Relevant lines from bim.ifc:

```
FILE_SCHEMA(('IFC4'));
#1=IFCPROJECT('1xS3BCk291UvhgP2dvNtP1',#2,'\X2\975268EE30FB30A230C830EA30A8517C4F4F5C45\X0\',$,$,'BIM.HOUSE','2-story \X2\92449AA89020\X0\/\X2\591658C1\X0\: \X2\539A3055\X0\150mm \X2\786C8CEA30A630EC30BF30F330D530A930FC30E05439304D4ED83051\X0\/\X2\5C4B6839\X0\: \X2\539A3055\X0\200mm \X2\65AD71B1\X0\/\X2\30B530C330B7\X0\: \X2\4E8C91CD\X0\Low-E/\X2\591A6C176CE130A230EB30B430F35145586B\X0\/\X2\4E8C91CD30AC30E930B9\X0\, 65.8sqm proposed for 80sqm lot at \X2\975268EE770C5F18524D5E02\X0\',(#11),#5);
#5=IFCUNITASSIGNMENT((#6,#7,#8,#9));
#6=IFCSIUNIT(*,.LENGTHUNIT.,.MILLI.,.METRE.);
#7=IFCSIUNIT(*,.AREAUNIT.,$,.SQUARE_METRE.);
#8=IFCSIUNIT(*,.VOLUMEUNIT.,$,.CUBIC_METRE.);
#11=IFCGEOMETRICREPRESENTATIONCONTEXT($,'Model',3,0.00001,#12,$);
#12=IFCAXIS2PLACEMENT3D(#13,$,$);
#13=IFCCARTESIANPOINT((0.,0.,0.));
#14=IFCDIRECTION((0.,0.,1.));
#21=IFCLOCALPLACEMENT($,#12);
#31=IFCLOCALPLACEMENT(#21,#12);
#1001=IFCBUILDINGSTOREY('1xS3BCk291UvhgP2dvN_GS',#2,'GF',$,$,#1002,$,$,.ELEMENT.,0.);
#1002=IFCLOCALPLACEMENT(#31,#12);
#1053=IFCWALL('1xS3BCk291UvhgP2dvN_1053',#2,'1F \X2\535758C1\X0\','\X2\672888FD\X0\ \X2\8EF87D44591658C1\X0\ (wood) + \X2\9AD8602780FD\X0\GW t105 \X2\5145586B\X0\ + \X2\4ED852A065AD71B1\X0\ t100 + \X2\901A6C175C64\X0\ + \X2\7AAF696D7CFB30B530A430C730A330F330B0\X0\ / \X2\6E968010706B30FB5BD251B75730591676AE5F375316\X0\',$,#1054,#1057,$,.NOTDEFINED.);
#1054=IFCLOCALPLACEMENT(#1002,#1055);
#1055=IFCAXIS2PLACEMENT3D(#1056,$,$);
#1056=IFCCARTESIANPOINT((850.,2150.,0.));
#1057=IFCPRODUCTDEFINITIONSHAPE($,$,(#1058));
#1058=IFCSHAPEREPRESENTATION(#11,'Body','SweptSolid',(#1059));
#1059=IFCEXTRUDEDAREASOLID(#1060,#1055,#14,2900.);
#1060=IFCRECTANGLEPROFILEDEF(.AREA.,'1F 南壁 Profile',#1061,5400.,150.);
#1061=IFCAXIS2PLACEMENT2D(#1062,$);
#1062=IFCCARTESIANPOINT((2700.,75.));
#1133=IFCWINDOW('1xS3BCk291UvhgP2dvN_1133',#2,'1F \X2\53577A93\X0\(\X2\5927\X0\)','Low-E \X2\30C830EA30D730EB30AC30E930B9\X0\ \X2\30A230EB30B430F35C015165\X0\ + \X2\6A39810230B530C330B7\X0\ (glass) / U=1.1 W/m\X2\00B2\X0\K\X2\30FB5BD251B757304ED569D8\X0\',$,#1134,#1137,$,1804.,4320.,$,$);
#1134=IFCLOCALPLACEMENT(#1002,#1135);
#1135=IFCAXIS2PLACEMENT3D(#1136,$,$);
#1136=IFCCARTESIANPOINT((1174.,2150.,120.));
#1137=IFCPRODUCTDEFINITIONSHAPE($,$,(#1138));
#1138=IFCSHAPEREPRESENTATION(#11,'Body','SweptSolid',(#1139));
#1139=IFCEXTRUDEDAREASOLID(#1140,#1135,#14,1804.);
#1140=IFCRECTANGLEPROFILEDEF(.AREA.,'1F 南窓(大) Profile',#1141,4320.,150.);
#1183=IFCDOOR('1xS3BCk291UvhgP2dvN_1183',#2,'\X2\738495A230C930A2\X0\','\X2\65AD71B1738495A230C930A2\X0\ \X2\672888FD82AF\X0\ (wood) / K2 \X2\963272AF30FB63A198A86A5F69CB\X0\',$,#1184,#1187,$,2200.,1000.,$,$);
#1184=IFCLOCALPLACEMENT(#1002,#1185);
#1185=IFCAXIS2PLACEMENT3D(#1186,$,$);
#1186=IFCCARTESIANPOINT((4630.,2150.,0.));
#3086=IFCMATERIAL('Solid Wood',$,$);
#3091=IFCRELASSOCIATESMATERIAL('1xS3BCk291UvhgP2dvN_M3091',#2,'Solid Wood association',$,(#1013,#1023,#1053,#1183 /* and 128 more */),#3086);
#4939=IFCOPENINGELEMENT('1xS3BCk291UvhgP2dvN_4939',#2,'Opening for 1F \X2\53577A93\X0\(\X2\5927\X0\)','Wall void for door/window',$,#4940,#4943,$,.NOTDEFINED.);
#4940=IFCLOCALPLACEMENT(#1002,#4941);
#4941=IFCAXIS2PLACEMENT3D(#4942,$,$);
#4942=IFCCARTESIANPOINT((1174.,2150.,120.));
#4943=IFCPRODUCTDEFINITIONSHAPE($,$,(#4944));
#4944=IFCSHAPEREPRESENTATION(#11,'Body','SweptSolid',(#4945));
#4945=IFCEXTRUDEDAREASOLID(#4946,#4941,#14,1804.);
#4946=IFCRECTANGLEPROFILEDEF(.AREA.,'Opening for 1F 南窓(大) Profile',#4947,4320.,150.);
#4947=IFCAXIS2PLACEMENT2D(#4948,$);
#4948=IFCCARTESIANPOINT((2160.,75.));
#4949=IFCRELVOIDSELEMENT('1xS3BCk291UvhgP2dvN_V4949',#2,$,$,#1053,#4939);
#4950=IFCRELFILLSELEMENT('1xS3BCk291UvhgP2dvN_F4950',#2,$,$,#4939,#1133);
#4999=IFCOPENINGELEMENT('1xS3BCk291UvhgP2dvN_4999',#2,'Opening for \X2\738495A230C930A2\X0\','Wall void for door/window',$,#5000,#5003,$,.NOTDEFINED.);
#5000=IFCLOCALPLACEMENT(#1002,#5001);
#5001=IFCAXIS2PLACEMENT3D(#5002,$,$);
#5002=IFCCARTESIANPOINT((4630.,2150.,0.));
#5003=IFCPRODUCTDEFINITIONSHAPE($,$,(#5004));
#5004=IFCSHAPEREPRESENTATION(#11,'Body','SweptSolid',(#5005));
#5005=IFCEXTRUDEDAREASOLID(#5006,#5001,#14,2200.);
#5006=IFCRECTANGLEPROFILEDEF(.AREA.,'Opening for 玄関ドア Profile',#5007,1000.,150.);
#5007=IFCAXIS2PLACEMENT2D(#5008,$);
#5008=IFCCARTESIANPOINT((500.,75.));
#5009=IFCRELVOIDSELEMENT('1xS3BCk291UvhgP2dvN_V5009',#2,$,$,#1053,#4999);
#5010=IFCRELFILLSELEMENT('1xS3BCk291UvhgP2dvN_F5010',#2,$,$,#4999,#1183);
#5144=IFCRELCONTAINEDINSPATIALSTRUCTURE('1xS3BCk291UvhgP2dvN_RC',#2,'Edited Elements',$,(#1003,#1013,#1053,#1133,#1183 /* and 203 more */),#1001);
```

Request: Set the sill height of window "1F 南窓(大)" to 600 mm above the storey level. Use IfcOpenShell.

```python
import numpy as np
import ifcopenshell
import ifcopenshell.api.geometry
import ifcopenshell.geom
import ifcopenshell.util.element
import ifcopenshell.util.placement
import ifcopenshell.util.shape
import ifcopenshell.util.unit

model = ifcopenshell.open("bim.ifc")
unit_scale = ifcopenshell.util.unit.calculate_unit_scale(model)

window = model.by_guid("1xS3BCk291UvhgP2dvN_1133")
opening = window.FillsVoids[0].RelatingOpeningElement
storey = ifcopenshell.util.element.get_container(window, ifc_class="IfcBuildingStorey")
level = ifcopenshell.util.placement.get_local_placement(storey.ObjectPlacement)[2, 3]

# The opening's origin need not be at the sill, so measure its lowest point.
shape = ifcopenshell.geom.create_shape(ifcopenshell.geom.settings(), opening)
bottom = ifcopenshell.util.shape.get_shape_bottom_elevation(shape, shape.geometry) / unit_scale
dz = level + 600.0 - bottom

shift = np.array([0.0, 0.0, dz])
# The window is not placed relative to its opening, so move both.
for product in (opening, window):
    matrix = ifcopenshell.util.placement.get_local_placement(product.ObjectPlacement)
    matrix[:3, 3] += shift
    ifcopenshell.api.geometry.edit_object_placement(model, product=product, matrix=matrix, is_si=False)

print(f"moved by {dz * unit_scale:+.3f} m")

model.write("bim_v2.ifc")
```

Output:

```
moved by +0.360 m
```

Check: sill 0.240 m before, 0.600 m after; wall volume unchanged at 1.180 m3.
